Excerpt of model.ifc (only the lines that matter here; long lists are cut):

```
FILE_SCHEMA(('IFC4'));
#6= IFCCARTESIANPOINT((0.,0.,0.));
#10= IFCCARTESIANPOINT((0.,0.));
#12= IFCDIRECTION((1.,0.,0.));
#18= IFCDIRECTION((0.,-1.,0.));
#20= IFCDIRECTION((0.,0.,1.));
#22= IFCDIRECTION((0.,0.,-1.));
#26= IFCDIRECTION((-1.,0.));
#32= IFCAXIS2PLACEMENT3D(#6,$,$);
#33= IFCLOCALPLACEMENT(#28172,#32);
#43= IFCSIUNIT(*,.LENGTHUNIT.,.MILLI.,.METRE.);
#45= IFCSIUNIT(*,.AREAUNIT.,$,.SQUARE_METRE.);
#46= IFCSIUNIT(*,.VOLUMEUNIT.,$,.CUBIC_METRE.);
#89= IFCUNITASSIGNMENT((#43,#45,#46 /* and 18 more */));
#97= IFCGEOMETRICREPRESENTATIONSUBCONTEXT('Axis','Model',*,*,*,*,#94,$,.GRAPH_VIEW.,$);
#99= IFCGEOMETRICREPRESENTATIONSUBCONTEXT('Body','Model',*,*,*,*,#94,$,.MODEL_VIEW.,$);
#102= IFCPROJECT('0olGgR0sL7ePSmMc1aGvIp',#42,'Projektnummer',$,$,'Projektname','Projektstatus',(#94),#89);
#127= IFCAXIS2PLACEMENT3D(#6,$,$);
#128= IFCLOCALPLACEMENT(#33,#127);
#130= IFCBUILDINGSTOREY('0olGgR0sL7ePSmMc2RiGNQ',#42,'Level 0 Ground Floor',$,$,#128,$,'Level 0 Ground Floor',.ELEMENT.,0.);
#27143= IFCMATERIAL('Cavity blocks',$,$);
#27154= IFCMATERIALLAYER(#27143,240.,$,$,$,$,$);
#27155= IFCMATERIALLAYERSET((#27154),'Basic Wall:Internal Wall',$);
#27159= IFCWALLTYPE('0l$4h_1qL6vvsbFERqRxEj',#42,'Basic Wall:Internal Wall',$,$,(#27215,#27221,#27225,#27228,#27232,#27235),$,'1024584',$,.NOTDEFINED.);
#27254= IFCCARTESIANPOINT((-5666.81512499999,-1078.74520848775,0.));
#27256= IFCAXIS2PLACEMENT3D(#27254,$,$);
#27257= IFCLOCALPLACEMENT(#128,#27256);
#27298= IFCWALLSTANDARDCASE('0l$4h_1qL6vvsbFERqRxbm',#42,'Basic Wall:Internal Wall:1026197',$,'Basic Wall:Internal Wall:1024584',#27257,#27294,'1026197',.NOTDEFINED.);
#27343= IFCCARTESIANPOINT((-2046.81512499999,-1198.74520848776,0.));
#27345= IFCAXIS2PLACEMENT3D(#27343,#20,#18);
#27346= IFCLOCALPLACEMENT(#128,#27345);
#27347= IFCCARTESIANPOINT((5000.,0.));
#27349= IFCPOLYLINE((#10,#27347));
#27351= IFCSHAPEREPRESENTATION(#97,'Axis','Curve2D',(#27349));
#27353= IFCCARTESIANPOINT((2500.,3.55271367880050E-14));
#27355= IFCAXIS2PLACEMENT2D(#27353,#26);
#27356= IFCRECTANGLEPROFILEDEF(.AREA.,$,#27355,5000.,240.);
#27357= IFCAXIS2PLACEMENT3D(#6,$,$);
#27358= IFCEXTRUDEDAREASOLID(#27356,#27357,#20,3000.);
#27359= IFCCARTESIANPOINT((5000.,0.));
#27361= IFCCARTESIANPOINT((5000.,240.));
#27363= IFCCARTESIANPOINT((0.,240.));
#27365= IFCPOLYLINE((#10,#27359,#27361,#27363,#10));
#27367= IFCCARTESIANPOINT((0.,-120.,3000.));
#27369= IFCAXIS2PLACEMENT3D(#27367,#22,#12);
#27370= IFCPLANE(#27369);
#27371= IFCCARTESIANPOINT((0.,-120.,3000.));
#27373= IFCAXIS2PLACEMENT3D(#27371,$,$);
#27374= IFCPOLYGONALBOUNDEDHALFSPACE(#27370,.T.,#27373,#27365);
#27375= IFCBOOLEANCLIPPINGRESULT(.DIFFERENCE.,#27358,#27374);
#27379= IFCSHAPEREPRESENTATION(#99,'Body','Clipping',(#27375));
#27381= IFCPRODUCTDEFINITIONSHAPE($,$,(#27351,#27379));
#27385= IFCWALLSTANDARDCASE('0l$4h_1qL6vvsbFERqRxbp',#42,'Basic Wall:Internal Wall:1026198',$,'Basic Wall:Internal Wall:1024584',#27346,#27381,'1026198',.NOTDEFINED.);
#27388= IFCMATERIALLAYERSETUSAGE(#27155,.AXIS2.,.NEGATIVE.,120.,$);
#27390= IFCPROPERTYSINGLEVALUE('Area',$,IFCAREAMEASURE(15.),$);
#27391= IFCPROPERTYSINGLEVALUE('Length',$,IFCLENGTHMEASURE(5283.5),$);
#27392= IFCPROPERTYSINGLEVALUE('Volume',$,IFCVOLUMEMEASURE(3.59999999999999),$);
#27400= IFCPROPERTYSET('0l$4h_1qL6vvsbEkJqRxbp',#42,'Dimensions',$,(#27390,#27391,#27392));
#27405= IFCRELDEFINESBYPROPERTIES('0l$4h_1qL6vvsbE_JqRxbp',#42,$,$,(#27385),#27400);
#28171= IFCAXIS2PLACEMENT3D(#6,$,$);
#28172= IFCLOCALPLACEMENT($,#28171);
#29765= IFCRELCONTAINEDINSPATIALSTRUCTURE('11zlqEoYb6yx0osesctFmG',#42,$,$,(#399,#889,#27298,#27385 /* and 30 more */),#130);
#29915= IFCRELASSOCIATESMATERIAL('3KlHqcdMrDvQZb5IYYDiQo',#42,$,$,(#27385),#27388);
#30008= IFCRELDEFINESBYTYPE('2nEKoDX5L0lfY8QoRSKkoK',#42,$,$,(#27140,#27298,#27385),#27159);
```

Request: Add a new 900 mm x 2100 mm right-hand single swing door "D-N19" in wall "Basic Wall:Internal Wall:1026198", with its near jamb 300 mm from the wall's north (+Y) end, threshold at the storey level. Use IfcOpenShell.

```python
import numpy as np
import ifcopenshell
import ifcopenshell.api.feature
import ifcopenshell.api.geometry
import ifcopenshell.api.pset
import ifcopenshell.api.root
import ifcopenshell.api.spatial
import ifcopenshell.geom
import ifcopenshell.util.element
import ifcopenshell.util.placement
import ifcopenshell.util.representation
import ifcopenshell.util.shape
import ifcopenshell.util.unit

model = ifcopenshell.open("model.ifc")
unit_scale = ifcopenshell.util.unit.calculate_unit_scale(model)
area_scale = ifcopenshell.util.unit.calculate_unit_scale(model, "AREAUNIT")
volume_scale = ifcopenshell.util.unit.calculate_unit_scale(model, "VOLUMEUNIT")
settings = ifcopenshell.geom.settings()


def volume(element):
    """Net volume in cubic metres, openings subtracted."""
    shape = ifcopenshell.geom.create_shape(settings, element)
    return ifcopenshell.util.shape.get_volume(shape.geometry)


wall = model.by_guid("0l$4h_1qL6vvsbFERqRxbp")
storey = ifcopenshell.util.element.get_container(wall, ifc_class="IfcBuildingStorey")
context = ifcopenshell.util.representation.get_context(model, "Model", "Body", "MODEL_VIEW")
before = volume(wall)

width, height, from_end, sill = 0.9, 2.1, 0.3, 0.0  # metres

# The wall runs along its own X axis, and the end named is its -X end.
wall_shape = ifcopenshell.geom.create_shape(settings, wall)
x, y, z = ifcopenshell.util.shape.get_vertices(wall_shape.geometry).T
start = x.min() + from_end
face, thickness = float(y.min()), float(y.max() - y.min())
wall_matrix = ifcopenshell.util.placement.get_local_placement(wall.ObjectPlacement)
level = ifcopenshell.util.placement.get_local_placement(storey.ObjectPlacement)[2, 3]


def in_wall(x, y):
    """Placement at x, y metres in the wall's axes, at sill height."""
    matrix = wall_matrix.copy()
    matrix[:, 3] = wall_matrix @ np.array([x / unit_scale, y / unit_scale, 0.0, 1.0])
    matrix[2, 3] = level + sill / unit_scale
    return matrix


# Opening: a box that overshoots both wall faces by 50 mm.
opening = ifcopenshell.api.root.create_entity(model, ifc_class="IfcOpeningElement", predefined_type="OPENING")
box = ifcopenshell.api.geometry.add_wall_representation(
    model, context=context, length=width, height=height, thickness=thickness + 0.1
)
ifcopenshell.api.geometry.assign_representation(model, product=opening, representation=box)
ifcopenshell.api.geometry.edit_object_placement(model, product=opening, matrix=in_wall(start, face - 0.05), is_si=False)
ifcopenshell.api.feature.add_feature(model, feature=opening, element=wall)

door = ifcopenshell.api.root.create_entity(model, ifc_class="IfcDoor", name="D-N19", predefined_type="DOOR")
door.OverallWidth, door.OverallHeight = width / unit_scale, height / unit_scale
door.OperationType = "SINGLE_SWING_RIGHT"
body = ifcopenshell.api.geometry.add_door_representation(
    model,
    context=context,
    overall_width=door.OverallWidth,
    overall_height=door.OverallHeight,
    operation_type="SINGLE_SWING_RIGHT",
    lining_properties={"LiningDepth": thickness / unit_scale, "ThresholdDepth": thickness / unit_scale},
)
ifcopenshell.api.geometry.assign_representation(model, product=door, representation=body)
ifcopenshell.api.spatial.assign_container(model, products=[door], relating_structure=storey)
ifcopenshell.api.feature.add_filling(model, opening=opening, element=door)

# The lining spans the wall, so the door starts at the wall face.
ifcopenshell.api.geometry.edit_object_placement(model, product=door, matrix=in_wall(start, face), is_si=False)

after = volume(wall)

# Update the wall's stored quantities.
pset = model.by_id(ifcopenshell.util.element.get_pset(wall, "Dimensions", should_inherit=False)["id"])
ifcopenshell.api.pset.edit_pset(model, pset=pset, properties={
    "Area": model.create_entity("IfcAreaMeasure", after / thickness / area_scale),
    "Volume": model.create_entity("IfcVolumeMeasure", after / volume_scale),
})

print(f"wall volume {before:.3f} -> {after:.3f} m3")

model.write("model_v2.ifc")
```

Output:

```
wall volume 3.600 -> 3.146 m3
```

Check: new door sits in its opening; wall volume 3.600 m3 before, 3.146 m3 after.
